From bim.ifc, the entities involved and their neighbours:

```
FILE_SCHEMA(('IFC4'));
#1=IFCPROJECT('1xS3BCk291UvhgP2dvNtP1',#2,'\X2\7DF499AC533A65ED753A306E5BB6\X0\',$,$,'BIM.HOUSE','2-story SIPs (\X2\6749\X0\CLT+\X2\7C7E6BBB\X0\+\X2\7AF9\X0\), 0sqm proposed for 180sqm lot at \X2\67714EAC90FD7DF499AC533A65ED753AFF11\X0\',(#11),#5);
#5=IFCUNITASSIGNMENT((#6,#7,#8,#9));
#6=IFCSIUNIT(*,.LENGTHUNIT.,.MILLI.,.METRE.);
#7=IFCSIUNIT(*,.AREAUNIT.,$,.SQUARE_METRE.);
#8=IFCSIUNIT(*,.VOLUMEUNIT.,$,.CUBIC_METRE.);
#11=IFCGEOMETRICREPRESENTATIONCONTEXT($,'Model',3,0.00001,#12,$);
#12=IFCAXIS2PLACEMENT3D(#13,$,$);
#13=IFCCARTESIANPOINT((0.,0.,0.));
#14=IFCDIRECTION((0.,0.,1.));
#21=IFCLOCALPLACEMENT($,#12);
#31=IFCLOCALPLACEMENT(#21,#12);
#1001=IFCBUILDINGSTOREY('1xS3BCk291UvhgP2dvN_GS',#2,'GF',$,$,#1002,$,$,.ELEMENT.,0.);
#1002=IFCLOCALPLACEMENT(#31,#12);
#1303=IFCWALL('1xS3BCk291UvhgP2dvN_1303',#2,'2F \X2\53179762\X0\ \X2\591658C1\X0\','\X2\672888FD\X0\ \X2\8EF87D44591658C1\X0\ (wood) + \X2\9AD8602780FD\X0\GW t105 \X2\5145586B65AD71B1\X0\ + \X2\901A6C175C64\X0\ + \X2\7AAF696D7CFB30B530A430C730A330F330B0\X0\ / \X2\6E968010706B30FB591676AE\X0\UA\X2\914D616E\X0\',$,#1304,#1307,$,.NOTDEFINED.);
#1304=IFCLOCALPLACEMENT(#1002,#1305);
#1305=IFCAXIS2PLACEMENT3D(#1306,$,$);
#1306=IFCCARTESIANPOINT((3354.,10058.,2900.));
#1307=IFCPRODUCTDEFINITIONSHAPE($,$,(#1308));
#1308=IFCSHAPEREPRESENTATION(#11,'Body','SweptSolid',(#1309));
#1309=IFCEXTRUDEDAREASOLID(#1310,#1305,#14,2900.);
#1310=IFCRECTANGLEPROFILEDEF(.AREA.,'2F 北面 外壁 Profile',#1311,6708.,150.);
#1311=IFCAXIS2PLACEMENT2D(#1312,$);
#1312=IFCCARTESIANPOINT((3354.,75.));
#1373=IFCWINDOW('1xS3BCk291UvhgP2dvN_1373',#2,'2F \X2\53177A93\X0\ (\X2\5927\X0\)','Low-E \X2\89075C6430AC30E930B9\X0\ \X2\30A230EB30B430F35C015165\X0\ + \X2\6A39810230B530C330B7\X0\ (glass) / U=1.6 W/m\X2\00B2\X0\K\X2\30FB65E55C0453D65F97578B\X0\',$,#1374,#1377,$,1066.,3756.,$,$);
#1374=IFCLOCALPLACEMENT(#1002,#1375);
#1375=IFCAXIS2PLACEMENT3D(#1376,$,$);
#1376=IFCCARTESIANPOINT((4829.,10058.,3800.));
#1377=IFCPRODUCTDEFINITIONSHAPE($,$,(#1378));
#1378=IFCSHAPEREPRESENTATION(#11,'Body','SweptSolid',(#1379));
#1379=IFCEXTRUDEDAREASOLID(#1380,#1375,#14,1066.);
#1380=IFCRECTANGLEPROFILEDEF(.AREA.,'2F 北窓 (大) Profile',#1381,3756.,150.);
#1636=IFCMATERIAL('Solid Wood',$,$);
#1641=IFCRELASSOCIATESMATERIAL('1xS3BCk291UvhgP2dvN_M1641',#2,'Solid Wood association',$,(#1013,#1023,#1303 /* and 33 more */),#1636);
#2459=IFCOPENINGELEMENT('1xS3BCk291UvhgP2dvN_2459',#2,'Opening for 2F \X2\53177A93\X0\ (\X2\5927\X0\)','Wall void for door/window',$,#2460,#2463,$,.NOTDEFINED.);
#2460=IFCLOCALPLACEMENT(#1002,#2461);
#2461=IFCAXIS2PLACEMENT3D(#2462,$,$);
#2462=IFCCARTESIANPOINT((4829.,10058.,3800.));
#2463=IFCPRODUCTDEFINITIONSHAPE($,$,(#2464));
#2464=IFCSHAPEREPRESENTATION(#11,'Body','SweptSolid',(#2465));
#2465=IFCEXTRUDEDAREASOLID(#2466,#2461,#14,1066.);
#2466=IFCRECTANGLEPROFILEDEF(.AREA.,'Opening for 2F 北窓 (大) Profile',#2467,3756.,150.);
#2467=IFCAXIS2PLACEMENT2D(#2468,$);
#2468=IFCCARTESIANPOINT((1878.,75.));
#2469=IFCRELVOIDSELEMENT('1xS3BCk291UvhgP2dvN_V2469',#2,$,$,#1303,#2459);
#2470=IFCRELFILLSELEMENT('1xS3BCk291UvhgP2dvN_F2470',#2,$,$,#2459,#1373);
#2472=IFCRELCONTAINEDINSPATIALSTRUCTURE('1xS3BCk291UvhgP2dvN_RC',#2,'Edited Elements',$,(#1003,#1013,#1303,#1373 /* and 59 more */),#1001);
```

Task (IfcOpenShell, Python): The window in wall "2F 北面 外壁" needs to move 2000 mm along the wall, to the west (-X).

```python
import ifcopenshell
import ifcopenshell.api.geometry
import ifcopenshell.util.placement
import ifcopenshell.util.unit

model = ifcopenshell.open("bim.ifc")
unit_scale = ifcopenshell.util.unit.calculate_unit_scale(model)

window = model.by_guid("1xS3BCk291UvhgP2dvN_1373")
opening = window.FillsVoids[0].RelatingOpeningElement
wall = opening.VoidsElements[0].RelatingBuildingElement

wall_matrix = ifcopenshell.util.placement.get_local_placement(wall.ObjectPlacement)
shift = wall_matrix[:3, 0] * -2 / unit_scale
before = ifcopenshell.util.placement.get_local_placement(window.ObjectPlacement)[:3, 3].copy()

# The window is not placed relative to its opening, so move both.
for product in (opening, window):
    matrix = ifcopenshell.util.placement.get_local_placement(product.ObjectPlacement)
    matrix[:3, 3] += shift
    ifcopenshell.api.geometry.edit_object_placement(model, product=product, matrix=matrix, is_si=False)

after = ifcopenshell.util.placement.get_local_placement(window.ObjectPlacement)[:3, 3]
print("window moved by", (after - before).round(3) + 0.0)

model.write("bim_edited.ifc")
```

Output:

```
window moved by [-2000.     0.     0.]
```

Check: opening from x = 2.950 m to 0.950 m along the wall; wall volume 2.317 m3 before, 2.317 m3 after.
